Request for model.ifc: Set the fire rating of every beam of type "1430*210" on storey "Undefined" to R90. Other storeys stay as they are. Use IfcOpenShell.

First a look at what the model holds.

```python
import ifcopenshell
import ifcopenshell.util.element

model = ifcopenshell.open("model.ifc")
print(model.schema)
storey = next(s for s in model.by_type("IfcBuildingStorey") if s.Name == "Undefined")
beams = [e for e in ifcopenshell.util.element.get_decomposition(storey) if e.is_a("IfcBeam")]
seen = {}
for e in beams:
    element_type = ifcopenshell.util.element.get_type(e)
    key = (element_type.Name if element_type != e and element_type else None, ifcopenshell.util.element.get_pset(e, "Pset_BeamCommon", "FireRating"))
    seen[key] = seen.get(key, 0) + 1
for (name, value), count in sorted(seen.items(), key=str):
    print(count, "x", name, "|", value)
```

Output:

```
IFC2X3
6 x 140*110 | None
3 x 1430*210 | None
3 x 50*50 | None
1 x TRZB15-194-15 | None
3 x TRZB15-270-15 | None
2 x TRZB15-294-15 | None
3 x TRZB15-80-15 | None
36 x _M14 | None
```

```python
import ifcopenshell
import ifcopenshell.api.pset
import ifcopenshell.util.element

model = ifcopenshell.open("model.ifc")

storey = next(s for s in model.by_type("IfcBuildingStorey") if s.Name == "Undefined")
beams = [e for e in ifcopenshell.util.element.get_decomposition(storey) if e.is_a("IfcBeam")]

count = 0
for e in beams:
    element_type = ifcopenshell.util.element.get_type(e)
    if element_type in (None, e) or element_type.Name != "1430*210":
        continue
    # add_pset returns the element's existing set when there is one.
    pset = ifcopenshell.api.pset.add_pset(model, product=e, name="Pset_BeamCommon")
    ifcopenshell.api.pset.edit_pset(model, pset=pset, properties={"FireRating": "R90"})
    count += 1

print(count, "beams updated")

model.write("model_v2.ifc")
```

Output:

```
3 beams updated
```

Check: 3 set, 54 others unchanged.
